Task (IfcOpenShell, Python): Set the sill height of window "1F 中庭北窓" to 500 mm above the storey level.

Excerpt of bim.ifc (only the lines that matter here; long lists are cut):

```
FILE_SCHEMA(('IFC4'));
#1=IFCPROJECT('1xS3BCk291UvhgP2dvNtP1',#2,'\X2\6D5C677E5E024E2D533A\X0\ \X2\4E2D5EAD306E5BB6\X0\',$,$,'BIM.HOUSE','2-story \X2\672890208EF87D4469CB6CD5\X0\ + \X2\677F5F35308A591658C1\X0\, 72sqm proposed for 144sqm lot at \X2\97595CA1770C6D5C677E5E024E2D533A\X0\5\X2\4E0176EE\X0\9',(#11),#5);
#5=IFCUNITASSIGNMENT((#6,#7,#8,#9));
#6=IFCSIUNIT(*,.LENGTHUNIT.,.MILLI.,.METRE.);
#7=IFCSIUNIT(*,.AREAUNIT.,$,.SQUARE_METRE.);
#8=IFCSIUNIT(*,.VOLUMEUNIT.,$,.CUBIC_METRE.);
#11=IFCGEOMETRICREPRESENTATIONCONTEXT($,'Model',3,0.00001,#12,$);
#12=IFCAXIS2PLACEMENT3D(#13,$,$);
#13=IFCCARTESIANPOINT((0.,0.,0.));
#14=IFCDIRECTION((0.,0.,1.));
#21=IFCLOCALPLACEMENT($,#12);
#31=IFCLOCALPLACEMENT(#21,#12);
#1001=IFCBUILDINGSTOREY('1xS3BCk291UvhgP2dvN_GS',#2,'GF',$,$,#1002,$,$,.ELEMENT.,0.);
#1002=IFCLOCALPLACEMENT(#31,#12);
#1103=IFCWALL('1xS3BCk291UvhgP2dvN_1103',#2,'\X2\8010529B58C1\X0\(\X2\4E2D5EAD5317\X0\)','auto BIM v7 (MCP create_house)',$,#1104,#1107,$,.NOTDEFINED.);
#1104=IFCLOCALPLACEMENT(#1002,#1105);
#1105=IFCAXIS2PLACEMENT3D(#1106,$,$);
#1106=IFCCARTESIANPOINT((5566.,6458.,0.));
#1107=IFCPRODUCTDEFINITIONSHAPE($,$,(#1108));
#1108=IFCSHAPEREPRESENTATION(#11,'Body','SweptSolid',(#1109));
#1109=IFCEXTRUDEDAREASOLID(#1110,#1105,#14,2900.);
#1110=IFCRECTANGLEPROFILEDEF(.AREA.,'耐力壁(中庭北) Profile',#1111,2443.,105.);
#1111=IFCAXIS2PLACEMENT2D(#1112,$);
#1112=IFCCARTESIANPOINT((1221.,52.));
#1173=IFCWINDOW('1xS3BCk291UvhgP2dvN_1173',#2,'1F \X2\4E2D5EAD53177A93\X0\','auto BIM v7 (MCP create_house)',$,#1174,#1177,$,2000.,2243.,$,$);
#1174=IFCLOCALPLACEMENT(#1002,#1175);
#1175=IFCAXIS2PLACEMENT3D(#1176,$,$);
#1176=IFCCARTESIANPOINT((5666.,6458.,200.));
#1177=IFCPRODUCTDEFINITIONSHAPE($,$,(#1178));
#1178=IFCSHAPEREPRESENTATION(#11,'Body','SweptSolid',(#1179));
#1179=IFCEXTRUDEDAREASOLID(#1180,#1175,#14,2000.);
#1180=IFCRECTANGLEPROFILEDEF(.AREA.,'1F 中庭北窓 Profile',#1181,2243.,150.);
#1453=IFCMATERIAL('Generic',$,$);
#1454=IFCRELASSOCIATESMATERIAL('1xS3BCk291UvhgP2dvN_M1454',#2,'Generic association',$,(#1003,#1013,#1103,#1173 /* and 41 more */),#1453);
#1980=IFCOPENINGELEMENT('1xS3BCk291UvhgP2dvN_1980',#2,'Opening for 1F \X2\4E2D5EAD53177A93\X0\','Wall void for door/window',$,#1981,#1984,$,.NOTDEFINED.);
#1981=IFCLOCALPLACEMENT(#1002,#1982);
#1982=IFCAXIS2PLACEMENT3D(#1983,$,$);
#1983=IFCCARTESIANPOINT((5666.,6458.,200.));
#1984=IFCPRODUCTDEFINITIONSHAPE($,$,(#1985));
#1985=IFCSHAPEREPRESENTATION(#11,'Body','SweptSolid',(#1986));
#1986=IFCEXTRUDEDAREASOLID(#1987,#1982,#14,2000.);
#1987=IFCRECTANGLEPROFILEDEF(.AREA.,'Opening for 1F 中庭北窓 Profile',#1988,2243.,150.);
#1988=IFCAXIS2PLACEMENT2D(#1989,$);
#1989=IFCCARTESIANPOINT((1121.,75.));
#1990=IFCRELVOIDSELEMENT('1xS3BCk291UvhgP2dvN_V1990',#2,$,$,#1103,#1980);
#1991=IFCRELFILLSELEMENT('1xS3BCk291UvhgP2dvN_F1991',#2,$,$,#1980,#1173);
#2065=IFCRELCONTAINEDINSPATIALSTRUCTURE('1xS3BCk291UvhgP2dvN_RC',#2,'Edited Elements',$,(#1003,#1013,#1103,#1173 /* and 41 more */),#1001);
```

```python
import numpy as np
import ifcopenshell
import ifcopenshell.api.geometry
import ifcopenshell.geom
import ifcopenshell.util.element
import ifcopenshell.util.placement
import ifcopenshell.util.shape
import ifcopenshell.util.unit

model = ifcopenshell.open("bim.ifc")
unit_scale = ifcopenshell.util.unit.calculate_unit_scale(model)

window = model.by_guid("1xS3BCk291UvhgP2dvN_1173")
opening = window.FillsVoids[0].RelatingOpeningElement
storey = ifcopenshell.util.element.get_container(window, ifc_class="IfcBuildingStorey")
level = ifcopenshell.util.placement.get_local_placement(storey.ObjectPlacement)[2, 3]

# The opening's origin need not be at the sill, so measure its lowest point.
shape = ifcopenshell.geom.create_shape(ifcopenshell.geom.settings(), opening)
bottom = ifcopenshell.util.shape.get_shape_bottom_elevation(shape, shape.geometry) / unit_scale
dz = level + 500.0 - bottom

shift = np.array([0.0, 0.0, dz])
# The window is not placed relative to its opening, so move both.
for product in (opening, window):
    matrix = ifcopenshell.util.placement.get_local_placement(product.ObjectPlacement)
    matrix[:3, 3] += shift
    ifcopenshell.api.geometry.edit_object_placement(model, product=product, matrix=matrix, is_si=False)

print(f"moved by {dz * unit_scale:+.3f} m")

model.write("bim_edited.ifc")
```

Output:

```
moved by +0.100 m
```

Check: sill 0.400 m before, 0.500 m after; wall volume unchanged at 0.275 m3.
